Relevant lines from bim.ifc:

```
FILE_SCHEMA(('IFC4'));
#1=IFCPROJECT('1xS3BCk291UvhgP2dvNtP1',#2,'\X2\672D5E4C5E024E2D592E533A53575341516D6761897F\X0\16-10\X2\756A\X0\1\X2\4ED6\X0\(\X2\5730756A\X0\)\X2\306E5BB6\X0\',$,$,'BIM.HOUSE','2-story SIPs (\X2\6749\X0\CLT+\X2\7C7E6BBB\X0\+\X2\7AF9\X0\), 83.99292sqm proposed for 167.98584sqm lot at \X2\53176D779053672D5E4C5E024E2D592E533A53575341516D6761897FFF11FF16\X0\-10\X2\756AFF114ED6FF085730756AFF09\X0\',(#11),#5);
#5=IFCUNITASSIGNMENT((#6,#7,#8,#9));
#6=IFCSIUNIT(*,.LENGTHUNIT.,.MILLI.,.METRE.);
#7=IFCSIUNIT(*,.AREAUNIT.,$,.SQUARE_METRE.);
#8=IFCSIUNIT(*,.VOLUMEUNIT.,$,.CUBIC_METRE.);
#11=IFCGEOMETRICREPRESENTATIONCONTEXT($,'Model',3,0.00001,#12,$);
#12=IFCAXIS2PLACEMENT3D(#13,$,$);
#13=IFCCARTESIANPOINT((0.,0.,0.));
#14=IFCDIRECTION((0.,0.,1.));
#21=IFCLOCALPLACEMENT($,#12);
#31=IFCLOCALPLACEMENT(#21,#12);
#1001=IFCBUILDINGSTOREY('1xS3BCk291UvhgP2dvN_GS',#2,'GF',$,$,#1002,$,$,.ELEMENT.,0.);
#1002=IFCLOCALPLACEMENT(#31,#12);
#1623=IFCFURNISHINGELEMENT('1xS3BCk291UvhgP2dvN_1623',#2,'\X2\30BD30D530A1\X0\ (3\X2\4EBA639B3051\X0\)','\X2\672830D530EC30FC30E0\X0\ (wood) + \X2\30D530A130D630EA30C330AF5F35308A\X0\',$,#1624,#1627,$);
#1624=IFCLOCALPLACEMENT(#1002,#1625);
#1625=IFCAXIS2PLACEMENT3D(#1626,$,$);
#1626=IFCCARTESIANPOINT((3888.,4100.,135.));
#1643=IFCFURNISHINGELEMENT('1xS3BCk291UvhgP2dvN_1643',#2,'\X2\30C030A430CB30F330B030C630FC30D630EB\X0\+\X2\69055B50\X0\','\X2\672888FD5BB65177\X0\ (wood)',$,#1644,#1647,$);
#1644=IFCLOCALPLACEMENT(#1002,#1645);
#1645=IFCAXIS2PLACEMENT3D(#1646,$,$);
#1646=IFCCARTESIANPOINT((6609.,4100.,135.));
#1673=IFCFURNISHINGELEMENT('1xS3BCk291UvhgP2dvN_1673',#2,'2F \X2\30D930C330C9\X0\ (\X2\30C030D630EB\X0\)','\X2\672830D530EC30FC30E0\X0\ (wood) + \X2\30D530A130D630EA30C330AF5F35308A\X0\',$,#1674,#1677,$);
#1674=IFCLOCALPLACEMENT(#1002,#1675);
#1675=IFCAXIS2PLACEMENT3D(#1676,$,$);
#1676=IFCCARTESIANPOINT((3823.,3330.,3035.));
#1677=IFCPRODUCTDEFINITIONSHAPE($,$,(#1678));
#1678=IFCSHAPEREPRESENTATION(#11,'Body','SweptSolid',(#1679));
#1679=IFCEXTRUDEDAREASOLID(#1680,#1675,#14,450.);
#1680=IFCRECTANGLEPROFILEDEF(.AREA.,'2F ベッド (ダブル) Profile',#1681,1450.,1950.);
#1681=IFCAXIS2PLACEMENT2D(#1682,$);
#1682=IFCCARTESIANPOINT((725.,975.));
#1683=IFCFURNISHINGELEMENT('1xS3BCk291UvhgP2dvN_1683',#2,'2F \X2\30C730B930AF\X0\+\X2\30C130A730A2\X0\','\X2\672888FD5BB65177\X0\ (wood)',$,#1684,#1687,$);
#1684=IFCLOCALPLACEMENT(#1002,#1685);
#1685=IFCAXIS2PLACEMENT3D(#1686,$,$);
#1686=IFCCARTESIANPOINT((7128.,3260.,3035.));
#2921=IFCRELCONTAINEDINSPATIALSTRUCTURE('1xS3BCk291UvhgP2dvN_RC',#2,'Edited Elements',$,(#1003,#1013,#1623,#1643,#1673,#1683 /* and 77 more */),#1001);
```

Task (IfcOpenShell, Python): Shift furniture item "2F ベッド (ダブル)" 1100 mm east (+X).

```python
import ifcopenshell
import ifcopenshell.api.geometry
import ifcopenshell.util.placement

model = ifcopenshell.open("bim.ifc")

item = model.by_id(1673)
matrix = ifcopenshell.util.placement.get_local_placement(item.ObjectPlacement)
matrix[0, 3] += 1100.0
ifcopenshell.api.geometry.edit_object_placement(model, product=item, matrix=matrix, is_si=False)

print(ifcopenshell.util.placement.get_local_placement(item.ObjectPlacement).round(3) + 0.0)

model.write("bim_updated.ifc")
```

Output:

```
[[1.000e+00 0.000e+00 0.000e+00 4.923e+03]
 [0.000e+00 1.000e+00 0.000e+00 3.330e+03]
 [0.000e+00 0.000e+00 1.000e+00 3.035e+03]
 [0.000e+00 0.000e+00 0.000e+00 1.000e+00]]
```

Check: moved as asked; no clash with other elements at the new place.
